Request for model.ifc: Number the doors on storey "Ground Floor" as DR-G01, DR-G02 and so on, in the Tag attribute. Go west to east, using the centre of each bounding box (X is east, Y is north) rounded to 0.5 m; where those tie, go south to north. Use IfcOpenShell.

First a look at what the model holds.

```python
import ifcopenshell
import ifcopenshell.util.element
import ifcopenshell.util.placement

model = ifcopenshell.open("model.ifc")
print(model.schema)
storey = next(s for s in model.by_type("IfcBuildingStorey") if s.Name == "Ground Floor")
doors = [e for e in ifcopenshell.util.element.get_decomposition(storey) if e.is_a("IfcDoor")]
for e in sorted(doors, key=lambda e: e.id()):
    origin = ifcopenshell.util.placement.get_local_placement(e.ObjectPlacement)[:3, 3]
    print(e.id(), e.Tag, e.Name, origin.round(2) + 0.0, sep=" | ")
```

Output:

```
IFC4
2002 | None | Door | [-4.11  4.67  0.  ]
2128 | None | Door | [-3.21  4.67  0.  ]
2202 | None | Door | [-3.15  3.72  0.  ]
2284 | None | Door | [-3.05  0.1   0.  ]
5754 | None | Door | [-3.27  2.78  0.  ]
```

```python
import ifcopenshell
import ifcopenshell.geom
import ifcopenshell.util.element
import ifcopenshell.util.shape

model = ifcopenshell.open("model.ifc")
settings = ifcopenshell.geom.settings()
settings.set("use-world-coords", True)


def centre(element):
    shape = ifcopenshell.geom.create_shape(settings, element)
    return ifcopenshell.util.shape.get_bbox_centroid(shape.geometry)


storey = next(s for s in model.by_type("IfcBuildingStorey") if s.Name == "Ground Floor")
doors = [e for e in ifcopenshell.util.element.get_decomposition(storey) if e.is_a("IfcDoor")]

# Insertion points can sit at a corner or the storey origin, so sort by the geometry (in metres).
centres = {e: centre(e) for e in doors}
doors.sort(key=lambda e: (round(centres[e][0] / 0.5), centres[e][1]))

for i, e in enumerate(doors, start=1):
    number = f"DR-G{i:02d}"
    e.Tag = number
    print(e.id(), number)

model.write("model_edited.ifc")
```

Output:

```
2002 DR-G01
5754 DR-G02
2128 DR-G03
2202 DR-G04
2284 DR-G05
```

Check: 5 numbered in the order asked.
